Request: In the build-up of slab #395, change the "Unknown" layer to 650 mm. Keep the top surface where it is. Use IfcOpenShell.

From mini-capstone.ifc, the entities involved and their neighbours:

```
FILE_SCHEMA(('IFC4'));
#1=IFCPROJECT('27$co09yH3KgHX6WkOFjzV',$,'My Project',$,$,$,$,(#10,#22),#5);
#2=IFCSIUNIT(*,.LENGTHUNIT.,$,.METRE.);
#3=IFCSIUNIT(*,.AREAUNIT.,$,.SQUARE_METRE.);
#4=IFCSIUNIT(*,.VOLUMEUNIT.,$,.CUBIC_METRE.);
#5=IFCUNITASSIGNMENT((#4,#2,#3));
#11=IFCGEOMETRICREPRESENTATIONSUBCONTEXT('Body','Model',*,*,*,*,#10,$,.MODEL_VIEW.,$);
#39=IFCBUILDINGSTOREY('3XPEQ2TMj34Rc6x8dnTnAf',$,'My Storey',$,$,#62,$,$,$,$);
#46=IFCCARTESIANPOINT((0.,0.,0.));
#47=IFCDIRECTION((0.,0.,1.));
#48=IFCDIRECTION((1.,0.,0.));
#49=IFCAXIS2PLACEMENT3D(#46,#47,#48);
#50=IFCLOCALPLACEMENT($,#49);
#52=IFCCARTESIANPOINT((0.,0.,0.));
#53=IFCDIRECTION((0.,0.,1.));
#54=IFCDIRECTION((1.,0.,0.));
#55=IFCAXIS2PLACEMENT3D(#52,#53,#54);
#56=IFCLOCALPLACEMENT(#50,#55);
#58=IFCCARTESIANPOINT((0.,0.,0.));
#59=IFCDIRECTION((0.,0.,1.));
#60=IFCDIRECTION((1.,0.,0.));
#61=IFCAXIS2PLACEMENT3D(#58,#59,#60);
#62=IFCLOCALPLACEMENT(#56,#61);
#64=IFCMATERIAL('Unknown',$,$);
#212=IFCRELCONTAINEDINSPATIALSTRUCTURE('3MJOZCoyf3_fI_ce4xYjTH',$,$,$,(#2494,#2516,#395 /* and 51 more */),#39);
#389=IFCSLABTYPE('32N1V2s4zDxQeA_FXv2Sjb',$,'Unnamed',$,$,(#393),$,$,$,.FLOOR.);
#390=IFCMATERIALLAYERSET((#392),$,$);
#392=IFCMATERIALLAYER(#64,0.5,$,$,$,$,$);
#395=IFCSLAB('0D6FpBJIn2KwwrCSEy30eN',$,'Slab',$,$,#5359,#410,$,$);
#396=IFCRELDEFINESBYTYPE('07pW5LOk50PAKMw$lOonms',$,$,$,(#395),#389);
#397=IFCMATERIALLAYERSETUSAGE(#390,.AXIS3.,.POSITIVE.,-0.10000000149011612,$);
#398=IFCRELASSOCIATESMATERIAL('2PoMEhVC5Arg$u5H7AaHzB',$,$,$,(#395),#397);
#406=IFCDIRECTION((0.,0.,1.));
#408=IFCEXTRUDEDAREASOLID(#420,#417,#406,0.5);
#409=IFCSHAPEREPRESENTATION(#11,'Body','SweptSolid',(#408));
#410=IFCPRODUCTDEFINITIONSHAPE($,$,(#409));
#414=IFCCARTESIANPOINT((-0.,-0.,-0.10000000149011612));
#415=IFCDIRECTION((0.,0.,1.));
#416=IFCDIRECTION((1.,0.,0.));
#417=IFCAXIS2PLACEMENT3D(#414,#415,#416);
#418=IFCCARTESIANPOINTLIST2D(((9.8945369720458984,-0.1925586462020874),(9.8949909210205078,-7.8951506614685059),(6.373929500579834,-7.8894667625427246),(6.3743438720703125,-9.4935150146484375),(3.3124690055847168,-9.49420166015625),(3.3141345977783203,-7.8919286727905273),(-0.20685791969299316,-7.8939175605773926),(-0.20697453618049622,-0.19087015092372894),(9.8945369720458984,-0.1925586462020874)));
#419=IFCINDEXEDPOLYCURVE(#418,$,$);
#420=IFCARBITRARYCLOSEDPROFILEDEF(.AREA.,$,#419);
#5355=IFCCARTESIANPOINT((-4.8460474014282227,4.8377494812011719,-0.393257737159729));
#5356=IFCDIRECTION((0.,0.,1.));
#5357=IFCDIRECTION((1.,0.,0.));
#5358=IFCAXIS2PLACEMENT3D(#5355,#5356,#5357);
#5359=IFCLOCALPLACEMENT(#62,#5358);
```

```python
import ifcopenshell
import ifcopenshell.util.element
import ifcopenshell.util.representation
import ifcopenshell.util.unit

model = ifcopenshell.open("mini-capstone.ifc")
unit_scale = ifcopenshell.util.unit.calculate_unit_scale(model)

layer_set = model.by_id(390)
layer = next(l for l in layer_set.MaterialLayers if l.Material and l.Material.Name == "Unknown")
change = 0.65 / unit_scale - layer.LayerThickness
layer.LayerThickness += change

# Geometry does not follow the layer set by itself.
slabs = [e for e in ifcopenshell.util.element.get_elements_by_material(model, layer_set) if e.is_a("IfcSlab")]
for slab in sorted(slabs, key=lambda e: e.id()):
    body = ifcopenshell.util.representation.get_representation(slab, "Model", "Body")
    solid = body.Items[0]
    old_depth = solid.Depth
    solid.Depth += change
    # Extruded upwards: lower the start of the extrusion so the top stays.
    x, y, z = solid.Position.Location.Coordinates
    solid.Position.Location = model.createIfcCartesianPoint((x, y, z - change))
    print(slab.id(), f"{old_depth:g} -> {solid.Depth:g}")

# The layers are counted up from the underside, which has moved.
for usage in {ifcopenshell.util.element.get_material(slab) for slab in slabs}:
    usage.OffsetFromReferenceLine -= change

model.write("mini-capstone_rev.ifc")
```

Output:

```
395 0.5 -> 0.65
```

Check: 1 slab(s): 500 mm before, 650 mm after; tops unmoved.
